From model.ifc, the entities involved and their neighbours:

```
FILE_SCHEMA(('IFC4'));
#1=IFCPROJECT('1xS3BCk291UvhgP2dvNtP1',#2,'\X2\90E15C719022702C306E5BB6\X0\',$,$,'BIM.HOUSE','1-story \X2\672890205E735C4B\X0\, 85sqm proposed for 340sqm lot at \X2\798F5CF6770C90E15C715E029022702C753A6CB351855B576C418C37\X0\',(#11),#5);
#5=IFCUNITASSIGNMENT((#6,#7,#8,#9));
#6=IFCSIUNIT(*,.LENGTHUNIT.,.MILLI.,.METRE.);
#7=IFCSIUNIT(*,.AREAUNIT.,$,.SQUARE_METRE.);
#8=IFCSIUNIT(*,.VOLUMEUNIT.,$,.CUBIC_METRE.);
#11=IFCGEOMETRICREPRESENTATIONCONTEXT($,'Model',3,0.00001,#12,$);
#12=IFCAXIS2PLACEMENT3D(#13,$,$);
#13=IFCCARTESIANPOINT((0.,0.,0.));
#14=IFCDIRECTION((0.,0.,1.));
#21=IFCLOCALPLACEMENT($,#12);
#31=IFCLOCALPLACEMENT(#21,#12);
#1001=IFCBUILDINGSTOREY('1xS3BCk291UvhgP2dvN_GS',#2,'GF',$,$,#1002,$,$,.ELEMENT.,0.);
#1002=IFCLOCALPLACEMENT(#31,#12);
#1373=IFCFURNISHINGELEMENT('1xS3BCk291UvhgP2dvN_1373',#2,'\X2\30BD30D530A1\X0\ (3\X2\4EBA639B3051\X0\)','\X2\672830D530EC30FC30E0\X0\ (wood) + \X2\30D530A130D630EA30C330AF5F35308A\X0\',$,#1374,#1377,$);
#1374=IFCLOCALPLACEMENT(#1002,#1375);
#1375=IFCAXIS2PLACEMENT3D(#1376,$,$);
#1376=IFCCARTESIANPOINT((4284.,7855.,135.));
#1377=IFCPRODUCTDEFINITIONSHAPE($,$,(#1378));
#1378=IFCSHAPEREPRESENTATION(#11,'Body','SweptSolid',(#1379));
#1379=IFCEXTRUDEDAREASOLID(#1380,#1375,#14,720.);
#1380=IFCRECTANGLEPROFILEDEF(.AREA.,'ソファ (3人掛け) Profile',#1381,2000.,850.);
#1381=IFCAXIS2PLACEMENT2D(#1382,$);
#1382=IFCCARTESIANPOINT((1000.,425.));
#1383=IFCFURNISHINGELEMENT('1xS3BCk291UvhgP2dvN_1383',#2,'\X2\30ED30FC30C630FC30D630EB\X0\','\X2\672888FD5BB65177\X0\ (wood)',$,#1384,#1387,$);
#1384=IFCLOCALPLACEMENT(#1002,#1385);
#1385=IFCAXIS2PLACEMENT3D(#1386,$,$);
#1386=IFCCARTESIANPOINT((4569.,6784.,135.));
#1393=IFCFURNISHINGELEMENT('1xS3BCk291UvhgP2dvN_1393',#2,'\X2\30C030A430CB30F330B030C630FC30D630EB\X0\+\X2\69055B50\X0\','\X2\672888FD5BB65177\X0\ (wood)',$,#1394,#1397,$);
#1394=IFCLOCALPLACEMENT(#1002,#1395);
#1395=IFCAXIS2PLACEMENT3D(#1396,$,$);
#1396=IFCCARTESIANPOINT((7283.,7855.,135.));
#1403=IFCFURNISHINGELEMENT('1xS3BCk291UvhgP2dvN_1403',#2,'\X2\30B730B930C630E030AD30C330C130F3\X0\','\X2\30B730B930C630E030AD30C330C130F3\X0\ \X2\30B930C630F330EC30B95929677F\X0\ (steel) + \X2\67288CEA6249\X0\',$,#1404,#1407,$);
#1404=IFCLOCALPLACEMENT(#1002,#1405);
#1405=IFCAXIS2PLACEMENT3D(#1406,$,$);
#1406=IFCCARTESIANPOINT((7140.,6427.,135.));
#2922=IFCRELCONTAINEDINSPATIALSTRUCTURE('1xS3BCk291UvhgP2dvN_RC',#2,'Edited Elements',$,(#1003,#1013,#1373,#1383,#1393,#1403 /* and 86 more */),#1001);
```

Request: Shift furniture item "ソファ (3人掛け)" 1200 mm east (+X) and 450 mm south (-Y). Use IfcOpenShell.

```python
import ifcopenshell
import ifcopenshell.api.geometry
import ifcopenshell.util.placement
import ifcopenshell.util.unit

model = ifcopenshell.open("model.ifc")
unit_scale = ifcopenshell.util.unit.calculate_unit_scale(model)

item = model.by_guid("1xS3BCk291UvhgP2dvN_1373")
matrix = ifcopenshell.util.placement.get_local_placement(item.ObjectPlacement)
matrix[0, 3] += 1.2 / unit_scale
matrix[1, 3] -= 0.45 / unit_scale
ifcopenshell.api.geometry.edit_object_placement(model, product=item, matrix=matrix, is_si=False)

print(ifcopenshell.util.placement.get_local_placement(item.ObjectPlacement).round(3) + 0.0)

model.write("model_edited.ifc")
```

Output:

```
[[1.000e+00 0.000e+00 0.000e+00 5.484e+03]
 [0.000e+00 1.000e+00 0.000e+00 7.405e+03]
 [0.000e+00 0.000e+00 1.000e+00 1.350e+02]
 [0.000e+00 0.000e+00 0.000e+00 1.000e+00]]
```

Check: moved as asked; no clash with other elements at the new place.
